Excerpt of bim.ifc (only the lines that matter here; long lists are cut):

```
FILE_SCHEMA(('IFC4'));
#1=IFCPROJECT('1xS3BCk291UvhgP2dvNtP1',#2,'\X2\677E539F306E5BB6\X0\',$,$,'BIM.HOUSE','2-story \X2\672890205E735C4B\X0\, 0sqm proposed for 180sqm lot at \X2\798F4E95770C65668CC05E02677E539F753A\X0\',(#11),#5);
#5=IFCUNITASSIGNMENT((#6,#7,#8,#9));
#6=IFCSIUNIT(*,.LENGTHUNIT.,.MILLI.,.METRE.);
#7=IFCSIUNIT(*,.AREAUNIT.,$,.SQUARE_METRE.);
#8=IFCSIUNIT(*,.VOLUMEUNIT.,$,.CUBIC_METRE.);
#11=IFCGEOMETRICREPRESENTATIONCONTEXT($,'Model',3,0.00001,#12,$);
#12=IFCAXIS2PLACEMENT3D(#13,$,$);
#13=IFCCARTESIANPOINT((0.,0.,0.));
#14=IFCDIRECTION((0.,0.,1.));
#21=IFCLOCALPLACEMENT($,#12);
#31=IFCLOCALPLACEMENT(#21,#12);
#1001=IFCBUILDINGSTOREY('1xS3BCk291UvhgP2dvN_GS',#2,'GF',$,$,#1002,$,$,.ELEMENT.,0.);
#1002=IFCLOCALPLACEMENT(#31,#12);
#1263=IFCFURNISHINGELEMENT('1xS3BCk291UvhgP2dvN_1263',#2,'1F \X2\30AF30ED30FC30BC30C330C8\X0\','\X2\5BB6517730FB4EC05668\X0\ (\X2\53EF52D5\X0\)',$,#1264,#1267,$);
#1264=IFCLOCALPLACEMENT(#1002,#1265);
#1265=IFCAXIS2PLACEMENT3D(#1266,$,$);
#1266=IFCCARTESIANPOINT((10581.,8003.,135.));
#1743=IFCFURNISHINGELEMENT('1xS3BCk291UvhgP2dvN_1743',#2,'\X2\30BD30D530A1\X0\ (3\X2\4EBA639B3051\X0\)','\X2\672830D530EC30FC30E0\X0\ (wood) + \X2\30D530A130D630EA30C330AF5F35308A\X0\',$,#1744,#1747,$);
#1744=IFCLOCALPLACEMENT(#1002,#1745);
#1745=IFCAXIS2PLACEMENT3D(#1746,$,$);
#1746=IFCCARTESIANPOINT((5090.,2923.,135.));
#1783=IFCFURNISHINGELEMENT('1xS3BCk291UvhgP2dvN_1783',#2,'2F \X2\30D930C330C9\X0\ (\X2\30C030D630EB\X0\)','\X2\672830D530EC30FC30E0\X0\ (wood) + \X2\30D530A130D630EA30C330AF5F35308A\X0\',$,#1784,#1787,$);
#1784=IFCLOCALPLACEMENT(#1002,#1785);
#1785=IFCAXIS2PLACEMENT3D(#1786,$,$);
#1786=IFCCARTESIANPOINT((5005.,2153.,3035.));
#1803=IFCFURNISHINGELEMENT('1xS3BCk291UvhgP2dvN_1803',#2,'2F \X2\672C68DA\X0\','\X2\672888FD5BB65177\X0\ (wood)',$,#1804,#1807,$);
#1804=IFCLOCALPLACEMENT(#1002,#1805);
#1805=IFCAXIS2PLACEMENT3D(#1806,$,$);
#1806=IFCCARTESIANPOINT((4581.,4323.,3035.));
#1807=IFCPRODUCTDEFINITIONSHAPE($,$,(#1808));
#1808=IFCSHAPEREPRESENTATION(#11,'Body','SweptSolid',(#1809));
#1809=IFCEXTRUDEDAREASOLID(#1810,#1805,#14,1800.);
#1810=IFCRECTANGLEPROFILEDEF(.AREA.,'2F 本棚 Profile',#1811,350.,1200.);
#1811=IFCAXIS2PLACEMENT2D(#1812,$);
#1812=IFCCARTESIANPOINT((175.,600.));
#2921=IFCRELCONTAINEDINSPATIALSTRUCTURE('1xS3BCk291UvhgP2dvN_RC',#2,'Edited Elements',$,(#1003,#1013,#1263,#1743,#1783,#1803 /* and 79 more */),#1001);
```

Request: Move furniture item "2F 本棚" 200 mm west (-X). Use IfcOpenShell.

```python
import ifcopenshell
import ifcopenshell.api.geometry
import ifcopenshell.util.placement
import ifcopenshell.util.unit

model = ifcopenshell.open("bim.ifc")
unit_scale = ifcopenshell.util.unit.calculate_unit_scale(model)

item = model.by_guid("1xS3BCk291UvhgP2dvN_1803")
matrix = ifcopenshell.util.placement.get_local_placement(item.ObjectPlacement)
matrix[0, 3] -= 0.2 / unit_scale
ifcopenshell.api.geometry.edit_object_placement(model, product=item, matrix=matrix, is_si=False)

print(ifcopenshell.util.placement.get_local_placement(item.ObjectPlacement).round(3) + 0.0)

model.write("bim-out.ifc")
```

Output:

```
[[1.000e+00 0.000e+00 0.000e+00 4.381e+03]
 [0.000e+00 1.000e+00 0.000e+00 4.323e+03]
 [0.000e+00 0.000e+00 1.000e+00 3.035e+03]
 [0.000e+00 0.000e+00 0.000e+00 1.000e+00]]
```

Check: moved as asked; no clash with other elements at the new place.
